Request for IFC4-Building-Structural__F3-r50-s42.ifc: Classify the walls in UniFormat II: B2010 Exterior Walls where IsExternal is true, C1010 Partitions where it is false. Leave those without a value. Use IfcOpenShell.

First a look at what the model holds.

```python
import ifcopenshell
import ifcopenshell.util.element

model = ifcopenshell.open("IFC4-Building-Structural__F3-r50-s42.ifc")
print(model.schema)
print("classifications:", [c.Name for c in model.by_type("IfcClassification")])
values = [ifcopenshell.util.element.get_pset(e, "Pset_WallCommon", "IsExternal") for e in model.by_type("IfcWall")]
for value in (True, False, None):
    print("IsExternal", value, values.count(value))
```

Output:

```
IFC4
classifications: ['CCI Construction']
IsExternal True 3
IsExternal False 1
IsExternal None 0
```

```python
import ifcopenshell
import ifcopenshell.api.classification
import ifcopenshell.util.element

model = ifcopenshell.open("IFC4-Building-Structural__F3-r50-s42.ifc")

system = ifcopenshell.api.classification.add_classification(model, classification="UniFormat II")

walls = model.by_type("IfcWall")
external = {e: ifcopenshell.util.element.get_pset(e, "Pset_WallCommon", "IsExternal") for e in walls}
for flag, code, name in ((True, "B2010", "Exterior Walls"), (False, "C1010", "Partitions")):
    products = [e for e in walls if external[e] is flag]
    ifcopenshell.api.classification.add_reference(
        model, products=products, classification=system, identification=code, name=name
    )
    print(code, len(products))

model.write("IFC4-Building-Structural__F3-r50-s42_updated.ifc")
```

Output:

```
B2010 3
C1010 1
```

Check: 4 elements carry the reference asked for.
